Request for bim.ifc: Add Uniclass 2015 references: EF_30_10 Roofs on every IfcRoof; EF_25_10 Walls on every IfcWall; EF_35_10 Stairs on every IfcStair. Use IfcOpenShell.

First a look at what the model holds.

```python
import ifcopenshell

model = ifcopenshell.open("bim.ifc")
print(model.schema)
print("classifications:", [c.Name for c in model.by_type("IfcClassification")])
for ifc_class in ("IfcDoor", "IfcRoof", "IfcStair", "IfcWall", "IfcWindow"):
    print(ifc_class, len(model.by_type(ifc_class)))
```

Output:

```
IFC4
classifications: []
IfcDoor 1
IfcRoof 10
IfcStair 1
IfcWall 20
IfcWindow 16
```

```python
import ifcopenshell
import ifcopenshell.api.classification

model = ifcopenshell.open("bim.ifc")

system = ifcopenshell.api.classification.add_classification(model, classification="Uniclass 2015")

codes = {
    "IfcRoof": ("EF_30_10", "Roofs"),
    "IfcWall": ("EF_25_10", "Walls"),
    "IfcStair": ("EF_35_10", "Stairs"),
}
for ifc_class, (code, name) in codes.items():
    products = model.by_type(ifc_class)
    ifcopenshell.api.classification.add_reference(
        model, products=products, classification=system, identification=code, name=name
    )
    print(code, len(products))

model.write("bim_v2.ifc")
```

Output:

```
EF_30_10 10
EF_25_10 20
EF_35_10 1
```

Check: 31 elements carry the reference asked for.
